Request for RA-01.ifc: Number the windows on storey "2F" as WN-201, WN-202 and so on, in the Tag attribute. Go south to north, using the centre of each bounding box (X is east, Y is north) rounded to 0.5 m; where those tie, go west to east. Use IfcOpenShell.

First a look at what the model holds.

```python
import ifcopenshell
import ifcopenshell.util.element
import ifcopenshell.util.placement

model = ifcopenshell.open("RA-01.ifc")
print(model.schema)
storey = next(s for s in model.by_type("IfcBuildingStorey") if s.Name == "2F")
windows = [e for e in ifcopenshell.util.element.get_decomposition(storey) if e.is_a("IfcWindow")]
for e in sorted(windows, key=lambda e: e.id()):
    origin = ifcopenshell.util.placement.get_local_placement(e.ObjectPlacement)[:3, 3]
    print(e.id(), e.Tag, e.Name, origin.round(2) + 0.0, sep=" | ")
```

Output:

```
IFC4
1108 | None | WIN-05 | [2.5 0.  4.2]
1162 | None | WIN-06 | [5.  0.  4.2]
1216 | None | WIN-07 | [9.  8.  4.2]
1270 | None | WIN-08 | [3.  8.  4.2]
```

```python
import ifcopenshell
import ifcopenshell.geom
import ifcopenshell.util.element
import ifcopenshell.util.shape

model = ifcopenshell.open("RA-01.ifc")
settings = ifcopenshell.geom.settings()
settings.set("use-world-coords", True)


def centre(element):
    shape = ifcopenshell.geom.create_shape(settings, element)
    return ifcopenshell.util.shape.get_bbox_centroid(shape.geometry)


storey = next(s for s in model.by_type("IfcBuildingStorey") if s.Name == "2F")
windows = [e for e in ifcopenshell.util.element.get_decomposition(storey) if e.is_a("IfcWindow")]

# Insertion points can sit at a corner or the storey origin, so sort by the geometry (in metres).
centres = {e: centre(e) for e in windows}
windows.sort(key=lambda e: (round(centres[e][1] / 0.5), centres[e][0]))

for i, e in enumerate(windows, start=1):
    number = f"WN-2{i:02d}"
    e.Tag = number
    print(e.id(), number)

model.write("RA-01_v2.ifc")
```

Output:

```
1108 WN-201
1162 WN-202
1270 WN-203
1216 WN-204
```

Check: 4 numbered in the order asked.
